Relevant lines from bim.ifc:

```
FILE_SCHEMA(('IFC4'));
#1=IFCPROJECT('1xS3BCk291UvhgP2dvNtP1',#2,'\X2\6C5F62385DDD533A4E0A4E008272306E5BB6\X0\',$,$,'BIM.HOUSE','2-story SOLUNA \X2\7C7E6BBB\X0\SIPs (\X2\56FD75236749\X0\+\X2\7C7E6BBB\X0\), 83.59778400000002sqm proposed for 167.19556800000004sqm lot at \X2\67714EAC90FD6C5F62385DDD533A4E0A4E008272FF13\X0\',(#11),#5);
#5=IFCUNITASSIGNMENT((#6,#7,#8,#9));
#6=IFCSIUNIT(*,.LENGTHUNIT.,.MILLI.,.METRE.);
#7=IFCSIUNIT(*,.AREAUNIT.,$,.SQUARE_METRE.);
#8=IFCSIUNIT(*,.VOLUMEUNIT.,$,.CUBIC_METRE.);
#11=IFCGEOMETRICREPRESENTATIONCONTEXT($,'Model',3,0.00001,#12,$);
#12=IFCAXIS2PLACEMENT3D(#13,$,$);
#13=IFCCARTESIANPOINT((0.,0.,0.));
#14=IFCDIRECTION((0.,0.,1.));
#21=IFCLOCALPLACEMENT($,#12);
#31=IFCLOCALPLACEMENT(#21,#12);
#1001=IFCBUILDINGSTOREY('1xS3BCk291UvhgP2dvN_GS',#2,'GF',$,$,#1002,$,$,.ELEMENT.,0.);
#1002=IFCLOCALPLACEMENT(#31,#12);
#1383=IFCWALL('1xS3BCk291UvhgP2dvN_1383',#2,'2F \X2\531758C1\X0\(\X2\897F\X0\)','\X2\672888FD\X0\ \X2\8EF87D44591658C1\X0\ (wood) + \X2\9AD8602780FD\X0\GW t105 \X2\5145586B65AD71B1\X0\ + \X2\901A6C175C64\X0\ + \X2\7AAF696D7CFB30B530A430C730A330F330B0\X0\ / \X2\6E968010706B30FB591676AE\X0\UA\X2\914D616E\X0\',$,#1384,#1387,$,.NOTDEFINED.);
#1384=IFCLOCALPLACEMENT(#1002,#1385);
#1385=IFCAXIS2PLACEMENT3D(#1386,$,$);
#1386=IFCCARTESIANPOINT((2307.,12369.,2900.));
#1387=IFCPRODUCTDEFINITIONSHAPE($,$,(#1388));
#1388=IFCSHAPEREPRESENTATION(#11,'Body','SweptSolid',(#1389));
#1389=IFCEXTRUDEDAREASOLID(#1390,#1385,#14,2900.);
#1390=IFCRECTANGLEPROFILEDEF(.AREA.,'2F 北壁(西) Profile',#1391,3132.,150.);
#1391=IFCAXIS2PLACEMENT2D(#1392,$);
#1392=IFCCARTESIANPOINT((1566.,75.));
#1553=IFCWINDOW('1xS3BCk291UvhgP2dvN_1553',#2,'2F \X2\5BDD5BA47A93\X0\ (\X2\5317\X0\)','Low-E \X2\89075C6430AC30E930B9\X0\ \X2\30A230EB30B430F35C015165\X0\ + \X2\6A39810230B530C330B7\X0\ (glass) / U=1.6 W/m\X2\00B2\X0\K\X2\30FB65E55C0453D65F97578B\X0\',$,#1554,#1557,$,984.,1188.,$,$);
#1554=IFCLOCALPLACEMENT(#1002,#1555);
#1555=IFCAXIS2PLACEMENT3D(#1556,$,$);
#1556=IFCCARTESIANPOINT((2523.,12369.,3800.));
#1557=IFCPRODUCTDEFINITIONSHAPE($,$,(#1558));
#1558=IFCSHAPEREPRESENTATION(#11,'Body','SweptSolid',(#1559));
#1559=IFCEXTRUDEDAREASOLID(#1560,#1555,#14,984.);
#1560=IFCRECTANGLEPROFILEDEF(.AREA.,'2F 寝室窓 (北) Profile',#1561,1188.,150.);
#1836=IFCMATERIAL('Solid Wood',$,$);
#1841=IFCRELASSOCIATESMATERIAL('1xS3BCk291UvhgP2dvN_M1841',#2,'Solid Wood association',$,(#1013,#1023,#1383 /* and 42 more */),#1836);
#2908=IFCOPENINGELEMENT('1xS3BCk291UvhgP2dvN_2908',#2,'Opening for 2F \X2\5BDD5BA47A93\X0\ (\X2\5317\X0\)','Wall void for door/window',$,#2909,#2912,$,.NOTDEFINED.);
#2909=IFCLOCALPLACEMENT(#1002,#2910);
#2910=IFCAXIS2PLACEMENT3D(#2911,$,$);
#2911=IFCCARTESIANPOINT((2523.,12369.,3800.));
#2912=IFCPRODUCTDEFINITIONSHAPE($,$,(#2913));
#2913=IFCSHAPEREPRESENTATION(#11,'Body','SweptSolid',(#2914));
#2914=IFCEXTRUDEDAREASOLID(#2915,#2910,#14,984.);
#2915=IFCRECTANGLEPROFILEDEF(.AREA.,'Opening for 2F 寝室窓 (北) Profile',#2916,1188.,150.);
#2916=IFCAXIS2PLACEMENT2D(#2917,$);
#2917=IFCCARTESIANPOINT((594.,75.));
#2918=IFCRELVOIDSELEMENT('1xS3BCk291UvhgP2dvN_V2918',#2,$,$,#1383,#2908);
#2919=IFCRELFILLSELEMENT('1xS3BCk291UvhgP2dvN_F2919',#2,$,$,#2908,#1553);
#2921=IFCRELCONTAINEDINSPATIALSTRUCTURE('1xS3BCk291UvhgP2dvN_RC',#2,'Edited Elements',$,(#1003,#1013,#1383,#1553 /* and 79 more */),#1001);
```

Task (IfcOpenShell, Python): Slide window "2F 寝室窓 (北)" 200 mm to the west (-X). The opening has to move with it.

```python
import ifcopenshell
import ifcopenshell.api.geometry
import ifcopenshell.util.placement

model = ifcopenshell.open("bim.ifc")

window = model.by_guid("1xS3BCk291UvhgP2dvN_1553")
opening = window.FillsVoids[0].RelatingOpeningElement
wall = opening.VoidsElements[0].RelatingBuildingElement

wall_matrix = ifcopenshell.util.placement.get_local_placement(wall.ObjectPlacement)
shift = wall_matrix[:3, 0] * -200.0
before = ifcopenshell.util.placement.get_local_placement(window.ObjectPlacement)[:3, 3].copy()

# The window is not placed relative to its opening, so move both.
for product in (opening, window):
    matrix = ifcopenshell.util.placement.get_local_placement(product.ObjectPlacement)
    matrix[:3, 3] += shift
    ifcopenshell.api.geometry.edit_object_placement(model, product=product, matrix=matrix, is_si=False)

after = ifcopenshell.util.placement.get_local_placement(window.ObjectPlacement)[:3, 3]
print("window moved by", (after - before).round(3) + 0.0)

model.write("bim-out.ifc")
```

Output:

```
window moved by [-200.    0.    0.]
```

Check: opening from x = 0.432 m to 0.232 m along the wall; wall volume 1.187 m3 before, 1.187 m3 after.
